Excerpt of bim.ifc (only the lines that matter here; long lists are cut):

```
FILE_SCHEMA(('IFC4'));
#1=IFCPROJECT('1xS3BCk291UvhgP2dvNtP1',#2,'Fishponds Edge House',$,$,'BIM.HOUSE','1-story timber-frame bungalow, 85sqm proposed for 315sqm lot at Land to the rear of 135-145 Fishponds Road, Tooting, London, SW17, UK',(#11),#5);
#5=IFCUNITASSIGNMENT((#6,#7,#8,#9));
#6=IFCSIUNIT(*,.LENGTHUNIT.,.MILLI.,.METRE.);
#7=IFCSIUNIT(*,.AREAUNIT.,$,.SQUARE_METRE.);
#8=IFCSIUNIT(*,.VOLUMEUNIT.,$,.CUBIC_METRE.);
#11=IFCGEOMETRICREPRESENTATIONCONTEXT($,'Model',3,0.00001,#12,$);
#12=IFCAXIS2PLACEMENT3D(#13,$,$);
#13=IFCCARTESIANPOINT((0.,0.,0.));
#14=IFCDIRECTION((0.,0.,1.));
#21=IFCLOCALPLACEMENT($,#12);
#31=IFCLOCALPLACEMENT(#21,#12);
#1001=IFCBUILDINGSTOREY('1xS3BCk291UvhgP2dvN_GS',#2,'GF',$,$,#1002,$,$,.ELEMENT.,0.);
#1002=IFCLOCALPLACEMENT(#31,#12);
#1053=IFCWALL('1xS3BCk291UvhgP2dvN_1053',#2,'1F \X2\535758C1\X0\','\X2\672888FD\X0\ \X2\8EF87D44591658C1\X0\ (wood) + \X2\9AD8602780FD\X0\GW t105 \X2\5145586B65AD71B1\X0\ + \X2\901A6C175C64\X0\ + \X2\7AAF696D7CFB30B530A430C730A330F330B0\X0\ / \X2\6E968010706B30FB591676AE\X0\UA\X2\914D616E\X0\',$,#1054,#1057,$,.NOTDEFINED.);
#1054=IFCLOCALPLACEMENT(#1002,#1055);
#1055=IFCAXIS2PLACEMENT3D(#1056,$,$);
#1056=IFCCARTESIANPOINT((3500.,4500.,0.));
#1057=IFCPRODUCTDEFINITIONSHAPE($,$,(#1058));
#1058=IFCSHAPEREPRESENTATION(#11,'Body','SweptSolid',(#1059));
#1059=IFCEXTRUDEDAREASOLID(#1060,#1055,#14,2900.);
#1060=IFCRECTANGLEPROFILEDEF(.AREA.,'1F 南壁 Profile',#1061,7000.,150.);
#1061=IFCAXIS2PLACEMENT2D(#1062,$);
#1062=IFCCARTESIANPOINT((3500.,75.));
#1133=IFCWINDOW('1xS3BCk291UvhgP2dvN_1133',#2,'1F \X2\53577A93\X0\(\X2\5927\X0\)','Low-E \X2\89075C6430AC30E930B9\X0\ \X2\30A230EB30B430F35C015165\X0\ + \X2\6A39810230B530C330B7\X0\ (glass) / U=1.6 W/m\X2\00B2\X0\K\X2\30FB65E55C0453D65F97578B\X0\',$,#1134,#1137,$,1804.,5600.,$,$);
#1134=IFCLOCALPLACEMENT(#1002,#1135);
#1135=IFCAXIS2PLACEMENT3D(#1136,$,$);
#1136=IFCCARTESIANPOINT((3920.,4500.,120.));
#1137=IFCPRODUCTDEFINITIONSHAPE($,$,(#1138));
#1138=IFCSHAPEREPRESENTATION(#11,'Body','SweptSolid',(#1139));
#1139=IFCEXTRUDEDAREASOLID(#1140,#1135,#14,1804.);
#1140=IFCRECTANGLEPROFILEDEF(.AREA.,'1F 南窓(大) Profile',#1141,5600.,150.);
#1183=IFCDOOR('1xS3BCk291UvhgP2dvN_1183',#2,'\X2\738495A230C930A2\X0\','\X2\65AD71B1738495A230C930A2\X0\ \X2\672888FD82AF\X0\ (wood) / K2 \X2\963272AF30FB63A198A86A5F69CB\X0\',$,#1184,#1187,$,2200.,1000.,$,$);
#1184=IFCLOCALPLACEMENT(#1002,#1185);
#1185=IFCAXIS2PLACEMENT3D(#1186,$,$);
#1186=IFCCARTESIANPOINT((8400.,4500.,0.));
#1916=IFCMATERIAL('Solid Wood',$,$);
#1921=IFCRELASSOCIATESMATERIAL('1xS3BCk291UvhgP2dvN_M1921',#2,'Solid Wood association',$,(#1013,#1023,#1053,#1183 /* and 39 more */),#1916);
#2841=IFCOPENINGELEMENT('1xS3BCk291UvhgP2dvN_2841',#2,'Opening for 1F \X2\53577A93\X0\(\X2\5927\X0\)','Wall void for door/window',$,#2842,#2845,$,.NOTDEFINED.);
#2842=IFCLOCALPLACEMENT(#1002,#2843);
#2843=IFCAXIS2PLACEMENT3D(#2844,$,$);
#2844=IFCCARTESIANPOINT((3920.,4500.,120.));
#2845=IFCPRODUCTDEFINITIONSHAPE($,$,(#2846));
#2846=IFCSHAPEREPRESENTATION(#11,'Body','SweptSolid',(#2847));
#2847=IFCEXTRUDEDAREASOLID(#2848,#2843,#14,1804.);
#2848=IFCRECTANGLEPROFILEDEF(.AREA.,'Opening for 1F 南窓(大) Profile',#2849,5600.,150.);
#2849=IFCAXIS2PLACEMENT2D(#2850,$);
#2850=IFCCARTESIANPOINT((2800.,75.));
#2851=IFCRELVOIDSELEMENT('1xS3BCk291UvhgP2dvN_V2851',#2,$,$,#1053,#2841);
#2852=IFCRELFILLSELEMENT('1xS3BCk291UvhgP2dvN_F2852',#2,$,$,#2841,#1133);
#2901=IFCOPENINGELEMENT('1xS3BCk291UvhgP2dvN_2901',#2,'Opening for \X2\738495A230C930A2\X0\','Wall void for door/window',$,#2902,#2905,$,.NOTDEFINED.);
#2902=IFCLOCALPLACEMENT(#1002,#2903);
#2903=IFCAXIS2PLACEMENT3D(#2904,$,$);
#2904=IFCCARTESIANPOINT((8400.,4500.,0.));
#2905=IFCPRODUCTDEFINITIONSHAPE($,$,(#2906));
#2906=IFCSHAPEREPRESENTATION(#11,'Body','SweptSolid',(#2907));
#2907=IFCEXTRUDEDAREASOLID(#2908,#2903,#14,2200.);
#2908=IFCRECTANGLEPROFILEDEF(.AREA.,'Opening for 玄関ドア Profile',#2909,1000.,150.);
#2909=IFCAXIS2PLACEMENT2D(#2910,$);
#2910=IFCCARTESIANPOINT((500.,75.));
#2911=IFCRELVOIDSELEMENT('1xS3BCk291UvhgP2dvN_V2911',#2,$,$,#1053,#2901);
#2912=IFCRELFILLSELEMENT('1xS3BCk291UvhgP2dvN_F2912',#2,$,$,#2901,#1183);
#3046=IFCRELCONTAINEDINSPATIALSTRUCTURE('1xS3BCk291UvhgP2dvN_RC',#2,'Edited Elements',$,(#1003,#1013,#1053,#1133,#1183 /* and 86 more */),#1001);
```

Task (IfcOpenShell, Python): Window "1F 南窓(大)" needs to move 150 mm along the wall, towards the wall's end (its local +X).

```python
import ifcopenshell
import ifcopenshell.api.geometry
import ifcopenshell.util.placement

model = ifcopenshell.open("bim.ifc")

window = model.by_guid("1xS3BCk291UvhgP2dvN_1133")
opening = window.FillsVoids[0].RelatingOpeningElement
wall = opening.VoidsElements[0].RelatingBuildingElement

wall_matrix = ifcopenshell.util.placement.get_local_placement(wall.ObjectPlacement)
shift = wall_matrix[:3, 0] * 150.0
before = ifcopenshell.util.placement.get_local_placement(window.ObjectPlacement)[:3, 3].copy()

# The window is not placed relative to its opening, so move both.
for product in (opening, window):
    matrix = ifcopenshell.util.placement.get_local_placement(product.ObjectPlacement)
    matrix[:3, 3] += shift
    ifcopenshell.api.geometry.edit_object_placement(model, product=product, matrix=matrix, is_si=False)

after = ifcopenshell.util.placement.get_local_placement(window.ObjectPlacement)[:3, 3]
print("window moved by", (after - before).round(3) + 0.0)

model.write("bim_rev.ifc")
```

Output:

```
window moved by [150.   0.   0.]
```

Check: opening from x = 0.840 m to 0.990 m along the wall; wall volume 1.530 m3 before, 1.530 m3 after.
